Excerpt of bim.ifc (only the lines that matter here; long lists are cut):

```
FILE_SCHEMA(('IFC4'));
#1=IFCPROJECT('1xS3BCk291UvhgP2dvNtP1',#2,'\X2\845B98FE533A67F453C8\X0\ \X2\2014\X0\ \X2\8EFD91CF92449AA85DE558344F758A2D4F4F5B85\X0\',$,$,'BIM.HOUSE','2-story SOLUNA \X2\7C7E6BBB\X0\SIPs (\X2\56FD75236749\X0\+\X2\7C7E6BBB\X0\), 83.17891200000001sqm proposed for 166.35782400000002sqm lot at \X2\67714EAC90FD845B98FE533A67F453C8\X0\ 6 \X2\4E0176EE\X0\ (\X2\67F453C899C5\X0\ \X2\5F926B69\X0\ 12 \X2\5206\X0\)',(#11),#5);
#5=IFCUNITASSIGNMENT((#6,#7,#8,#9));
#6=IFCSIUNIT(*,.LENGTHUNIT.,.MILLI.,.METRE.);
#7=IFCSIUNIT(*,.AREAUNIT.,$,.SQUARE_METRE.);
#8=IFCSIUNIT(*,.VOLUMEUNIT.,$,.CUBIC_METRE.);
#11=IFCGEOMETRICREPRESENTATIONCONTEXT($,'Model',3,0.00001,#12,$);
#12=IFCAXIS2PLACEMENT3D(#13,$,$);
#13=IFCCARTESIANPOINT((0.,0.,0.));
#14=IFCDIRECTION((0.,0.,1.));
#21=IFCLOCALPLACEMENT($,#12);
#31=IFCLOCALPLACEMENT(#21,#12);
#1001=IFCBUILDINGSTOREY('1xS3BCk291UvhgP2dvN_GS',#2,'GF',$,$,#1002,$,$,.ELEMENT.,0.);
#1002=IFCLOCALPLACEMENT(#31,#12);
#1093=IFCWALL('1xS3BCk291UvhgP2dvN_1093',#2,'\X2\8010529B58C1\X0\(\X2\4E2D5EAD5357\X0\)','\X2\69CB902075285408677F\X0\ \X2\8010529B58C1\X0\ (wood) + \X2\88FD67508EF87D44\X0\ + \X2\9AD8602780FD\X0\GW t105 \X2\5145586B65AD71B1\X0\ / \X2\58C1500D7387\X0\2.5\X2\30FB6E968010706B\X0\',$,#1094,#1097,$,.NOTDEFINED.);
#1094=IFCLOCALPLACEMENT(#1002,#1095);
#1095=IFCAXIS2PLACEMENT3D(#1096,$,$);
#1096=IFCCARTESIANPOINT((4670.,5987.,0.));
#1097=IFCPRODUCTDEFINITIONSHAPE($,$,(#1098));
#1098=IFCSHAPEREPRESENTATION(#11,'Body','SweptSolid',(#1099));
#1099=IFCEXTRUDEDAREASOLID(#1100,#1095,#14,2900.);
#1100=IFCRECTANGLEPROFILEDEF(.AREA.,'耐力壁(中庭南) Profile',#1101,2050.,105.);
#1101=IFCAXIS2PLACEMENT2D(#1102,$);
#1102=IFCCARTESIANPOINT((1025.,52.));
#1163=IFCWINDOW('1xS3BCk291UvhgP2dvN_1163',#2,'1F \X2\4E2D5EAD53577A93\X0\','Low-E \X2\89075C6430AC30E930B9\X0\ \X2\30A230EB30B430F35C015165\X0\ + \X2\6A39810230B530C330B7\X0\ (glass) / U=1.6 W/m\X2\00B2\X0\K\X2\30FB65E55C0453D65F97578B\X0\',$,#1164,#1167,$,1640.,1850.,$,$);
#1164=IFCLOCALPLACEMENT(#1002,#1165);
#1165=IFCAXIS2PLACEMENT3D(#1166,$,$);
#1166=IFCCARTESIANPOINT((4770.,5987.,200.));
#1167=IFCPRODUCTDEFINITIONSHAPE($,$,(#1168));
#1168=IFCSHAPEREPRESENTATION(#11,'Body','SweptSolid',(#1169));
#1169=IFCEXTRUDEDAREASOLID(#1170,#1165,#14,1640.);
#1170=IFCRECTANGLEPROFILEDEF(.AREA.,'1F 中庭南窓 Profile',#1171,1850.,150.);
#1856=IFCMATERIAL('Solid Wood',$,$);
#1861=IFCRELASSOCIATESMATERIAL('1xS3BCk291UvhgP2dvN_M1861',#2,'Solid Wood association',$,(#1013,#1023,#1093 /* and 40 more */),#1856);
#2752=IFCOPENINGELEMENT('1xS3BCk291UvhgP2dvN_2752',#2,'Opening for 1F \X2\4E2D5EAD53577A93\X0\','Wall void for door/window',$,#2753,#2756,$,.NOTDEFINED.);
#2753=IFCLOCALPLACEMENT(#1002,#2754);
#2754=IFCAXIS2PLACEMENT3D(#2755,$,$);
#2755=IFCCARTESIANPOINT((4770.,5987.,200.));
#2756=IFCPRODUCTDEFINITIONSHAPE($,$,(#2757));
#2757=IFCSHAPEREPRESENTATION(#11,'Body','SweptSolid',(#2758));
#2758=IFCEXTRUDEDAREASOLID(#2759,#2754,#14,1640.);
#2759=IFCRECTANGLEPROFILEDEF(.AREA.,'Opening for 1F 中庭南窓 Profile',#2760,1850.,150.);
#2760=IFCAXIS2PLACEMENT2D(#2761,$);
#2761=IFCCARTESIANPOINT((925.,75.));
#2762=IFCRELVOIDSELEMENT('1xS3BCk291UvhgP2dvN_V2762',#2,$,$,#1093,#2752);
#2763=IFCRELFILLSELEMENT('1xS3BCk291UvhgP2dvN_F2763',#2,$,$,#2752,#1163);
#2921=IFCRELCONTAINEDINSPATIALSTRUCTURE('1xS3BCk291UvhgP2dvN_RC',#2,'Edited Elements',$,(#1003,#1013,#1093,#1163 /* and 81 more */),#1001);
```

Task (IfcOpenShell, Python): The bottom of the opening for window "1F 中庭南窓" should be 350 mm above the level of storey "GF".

```python
import numpy as np
import ifcopenshell
import ifcopenshell.api.geometry
import ifcopenshell.geom
import ifcopenshell.util.element
import ifcopenshell.util.placement
import ifcopenshell.util.shape
import ifcopenshell.util.unit

model = ifcopenshell.open("bim.ifc")
unit_scale = ifcopenshell.util.unit.calculate_unit_scale(model)

window = model.by_guid("1xS3BCk291UvhgP2dvN_1163")
opening = window.FillsVoids[0].RelatingOpeningElement
storey = ifcopenshell.util.element.get_container(window, ifc_class="IfcBuildingStorey")
level = ifcopenshell.util.placement.get_local_placement(storey.ObjectPlacement)[2, 3]

# The opening's origin need not be at the sill, so measure its lowest point.
shape = ifcopenshell.geom.create_shape(ifcopenshell.geom.settings(), opening)
bottom = ifcopenshell.util.shape.get_shape_bottom_elevation(shape, shape.geometry) / unit_scale
dz = level + 0.35 / unit_scale - bottom

shift = np.array([0.0, 0.0, dz])
# The window is not placed relative to its opening, so move both.
for product in (opening, window):
    matrix = ifcopenshell.util.placement.get_local_placement(product.ObjectPlacement)
    matrix[:3, 3] += shift
    ifcopenshell.api.geometry.edit_object_placement(model, product=product, matrix=matrix, is_si=False)

print(f"moved by {dz * unit_scale:+.3f} m")

model.write("bim_edited.ifc")
```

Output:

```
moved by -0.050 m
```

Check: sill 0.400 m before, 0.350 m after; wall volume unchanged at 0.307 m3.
